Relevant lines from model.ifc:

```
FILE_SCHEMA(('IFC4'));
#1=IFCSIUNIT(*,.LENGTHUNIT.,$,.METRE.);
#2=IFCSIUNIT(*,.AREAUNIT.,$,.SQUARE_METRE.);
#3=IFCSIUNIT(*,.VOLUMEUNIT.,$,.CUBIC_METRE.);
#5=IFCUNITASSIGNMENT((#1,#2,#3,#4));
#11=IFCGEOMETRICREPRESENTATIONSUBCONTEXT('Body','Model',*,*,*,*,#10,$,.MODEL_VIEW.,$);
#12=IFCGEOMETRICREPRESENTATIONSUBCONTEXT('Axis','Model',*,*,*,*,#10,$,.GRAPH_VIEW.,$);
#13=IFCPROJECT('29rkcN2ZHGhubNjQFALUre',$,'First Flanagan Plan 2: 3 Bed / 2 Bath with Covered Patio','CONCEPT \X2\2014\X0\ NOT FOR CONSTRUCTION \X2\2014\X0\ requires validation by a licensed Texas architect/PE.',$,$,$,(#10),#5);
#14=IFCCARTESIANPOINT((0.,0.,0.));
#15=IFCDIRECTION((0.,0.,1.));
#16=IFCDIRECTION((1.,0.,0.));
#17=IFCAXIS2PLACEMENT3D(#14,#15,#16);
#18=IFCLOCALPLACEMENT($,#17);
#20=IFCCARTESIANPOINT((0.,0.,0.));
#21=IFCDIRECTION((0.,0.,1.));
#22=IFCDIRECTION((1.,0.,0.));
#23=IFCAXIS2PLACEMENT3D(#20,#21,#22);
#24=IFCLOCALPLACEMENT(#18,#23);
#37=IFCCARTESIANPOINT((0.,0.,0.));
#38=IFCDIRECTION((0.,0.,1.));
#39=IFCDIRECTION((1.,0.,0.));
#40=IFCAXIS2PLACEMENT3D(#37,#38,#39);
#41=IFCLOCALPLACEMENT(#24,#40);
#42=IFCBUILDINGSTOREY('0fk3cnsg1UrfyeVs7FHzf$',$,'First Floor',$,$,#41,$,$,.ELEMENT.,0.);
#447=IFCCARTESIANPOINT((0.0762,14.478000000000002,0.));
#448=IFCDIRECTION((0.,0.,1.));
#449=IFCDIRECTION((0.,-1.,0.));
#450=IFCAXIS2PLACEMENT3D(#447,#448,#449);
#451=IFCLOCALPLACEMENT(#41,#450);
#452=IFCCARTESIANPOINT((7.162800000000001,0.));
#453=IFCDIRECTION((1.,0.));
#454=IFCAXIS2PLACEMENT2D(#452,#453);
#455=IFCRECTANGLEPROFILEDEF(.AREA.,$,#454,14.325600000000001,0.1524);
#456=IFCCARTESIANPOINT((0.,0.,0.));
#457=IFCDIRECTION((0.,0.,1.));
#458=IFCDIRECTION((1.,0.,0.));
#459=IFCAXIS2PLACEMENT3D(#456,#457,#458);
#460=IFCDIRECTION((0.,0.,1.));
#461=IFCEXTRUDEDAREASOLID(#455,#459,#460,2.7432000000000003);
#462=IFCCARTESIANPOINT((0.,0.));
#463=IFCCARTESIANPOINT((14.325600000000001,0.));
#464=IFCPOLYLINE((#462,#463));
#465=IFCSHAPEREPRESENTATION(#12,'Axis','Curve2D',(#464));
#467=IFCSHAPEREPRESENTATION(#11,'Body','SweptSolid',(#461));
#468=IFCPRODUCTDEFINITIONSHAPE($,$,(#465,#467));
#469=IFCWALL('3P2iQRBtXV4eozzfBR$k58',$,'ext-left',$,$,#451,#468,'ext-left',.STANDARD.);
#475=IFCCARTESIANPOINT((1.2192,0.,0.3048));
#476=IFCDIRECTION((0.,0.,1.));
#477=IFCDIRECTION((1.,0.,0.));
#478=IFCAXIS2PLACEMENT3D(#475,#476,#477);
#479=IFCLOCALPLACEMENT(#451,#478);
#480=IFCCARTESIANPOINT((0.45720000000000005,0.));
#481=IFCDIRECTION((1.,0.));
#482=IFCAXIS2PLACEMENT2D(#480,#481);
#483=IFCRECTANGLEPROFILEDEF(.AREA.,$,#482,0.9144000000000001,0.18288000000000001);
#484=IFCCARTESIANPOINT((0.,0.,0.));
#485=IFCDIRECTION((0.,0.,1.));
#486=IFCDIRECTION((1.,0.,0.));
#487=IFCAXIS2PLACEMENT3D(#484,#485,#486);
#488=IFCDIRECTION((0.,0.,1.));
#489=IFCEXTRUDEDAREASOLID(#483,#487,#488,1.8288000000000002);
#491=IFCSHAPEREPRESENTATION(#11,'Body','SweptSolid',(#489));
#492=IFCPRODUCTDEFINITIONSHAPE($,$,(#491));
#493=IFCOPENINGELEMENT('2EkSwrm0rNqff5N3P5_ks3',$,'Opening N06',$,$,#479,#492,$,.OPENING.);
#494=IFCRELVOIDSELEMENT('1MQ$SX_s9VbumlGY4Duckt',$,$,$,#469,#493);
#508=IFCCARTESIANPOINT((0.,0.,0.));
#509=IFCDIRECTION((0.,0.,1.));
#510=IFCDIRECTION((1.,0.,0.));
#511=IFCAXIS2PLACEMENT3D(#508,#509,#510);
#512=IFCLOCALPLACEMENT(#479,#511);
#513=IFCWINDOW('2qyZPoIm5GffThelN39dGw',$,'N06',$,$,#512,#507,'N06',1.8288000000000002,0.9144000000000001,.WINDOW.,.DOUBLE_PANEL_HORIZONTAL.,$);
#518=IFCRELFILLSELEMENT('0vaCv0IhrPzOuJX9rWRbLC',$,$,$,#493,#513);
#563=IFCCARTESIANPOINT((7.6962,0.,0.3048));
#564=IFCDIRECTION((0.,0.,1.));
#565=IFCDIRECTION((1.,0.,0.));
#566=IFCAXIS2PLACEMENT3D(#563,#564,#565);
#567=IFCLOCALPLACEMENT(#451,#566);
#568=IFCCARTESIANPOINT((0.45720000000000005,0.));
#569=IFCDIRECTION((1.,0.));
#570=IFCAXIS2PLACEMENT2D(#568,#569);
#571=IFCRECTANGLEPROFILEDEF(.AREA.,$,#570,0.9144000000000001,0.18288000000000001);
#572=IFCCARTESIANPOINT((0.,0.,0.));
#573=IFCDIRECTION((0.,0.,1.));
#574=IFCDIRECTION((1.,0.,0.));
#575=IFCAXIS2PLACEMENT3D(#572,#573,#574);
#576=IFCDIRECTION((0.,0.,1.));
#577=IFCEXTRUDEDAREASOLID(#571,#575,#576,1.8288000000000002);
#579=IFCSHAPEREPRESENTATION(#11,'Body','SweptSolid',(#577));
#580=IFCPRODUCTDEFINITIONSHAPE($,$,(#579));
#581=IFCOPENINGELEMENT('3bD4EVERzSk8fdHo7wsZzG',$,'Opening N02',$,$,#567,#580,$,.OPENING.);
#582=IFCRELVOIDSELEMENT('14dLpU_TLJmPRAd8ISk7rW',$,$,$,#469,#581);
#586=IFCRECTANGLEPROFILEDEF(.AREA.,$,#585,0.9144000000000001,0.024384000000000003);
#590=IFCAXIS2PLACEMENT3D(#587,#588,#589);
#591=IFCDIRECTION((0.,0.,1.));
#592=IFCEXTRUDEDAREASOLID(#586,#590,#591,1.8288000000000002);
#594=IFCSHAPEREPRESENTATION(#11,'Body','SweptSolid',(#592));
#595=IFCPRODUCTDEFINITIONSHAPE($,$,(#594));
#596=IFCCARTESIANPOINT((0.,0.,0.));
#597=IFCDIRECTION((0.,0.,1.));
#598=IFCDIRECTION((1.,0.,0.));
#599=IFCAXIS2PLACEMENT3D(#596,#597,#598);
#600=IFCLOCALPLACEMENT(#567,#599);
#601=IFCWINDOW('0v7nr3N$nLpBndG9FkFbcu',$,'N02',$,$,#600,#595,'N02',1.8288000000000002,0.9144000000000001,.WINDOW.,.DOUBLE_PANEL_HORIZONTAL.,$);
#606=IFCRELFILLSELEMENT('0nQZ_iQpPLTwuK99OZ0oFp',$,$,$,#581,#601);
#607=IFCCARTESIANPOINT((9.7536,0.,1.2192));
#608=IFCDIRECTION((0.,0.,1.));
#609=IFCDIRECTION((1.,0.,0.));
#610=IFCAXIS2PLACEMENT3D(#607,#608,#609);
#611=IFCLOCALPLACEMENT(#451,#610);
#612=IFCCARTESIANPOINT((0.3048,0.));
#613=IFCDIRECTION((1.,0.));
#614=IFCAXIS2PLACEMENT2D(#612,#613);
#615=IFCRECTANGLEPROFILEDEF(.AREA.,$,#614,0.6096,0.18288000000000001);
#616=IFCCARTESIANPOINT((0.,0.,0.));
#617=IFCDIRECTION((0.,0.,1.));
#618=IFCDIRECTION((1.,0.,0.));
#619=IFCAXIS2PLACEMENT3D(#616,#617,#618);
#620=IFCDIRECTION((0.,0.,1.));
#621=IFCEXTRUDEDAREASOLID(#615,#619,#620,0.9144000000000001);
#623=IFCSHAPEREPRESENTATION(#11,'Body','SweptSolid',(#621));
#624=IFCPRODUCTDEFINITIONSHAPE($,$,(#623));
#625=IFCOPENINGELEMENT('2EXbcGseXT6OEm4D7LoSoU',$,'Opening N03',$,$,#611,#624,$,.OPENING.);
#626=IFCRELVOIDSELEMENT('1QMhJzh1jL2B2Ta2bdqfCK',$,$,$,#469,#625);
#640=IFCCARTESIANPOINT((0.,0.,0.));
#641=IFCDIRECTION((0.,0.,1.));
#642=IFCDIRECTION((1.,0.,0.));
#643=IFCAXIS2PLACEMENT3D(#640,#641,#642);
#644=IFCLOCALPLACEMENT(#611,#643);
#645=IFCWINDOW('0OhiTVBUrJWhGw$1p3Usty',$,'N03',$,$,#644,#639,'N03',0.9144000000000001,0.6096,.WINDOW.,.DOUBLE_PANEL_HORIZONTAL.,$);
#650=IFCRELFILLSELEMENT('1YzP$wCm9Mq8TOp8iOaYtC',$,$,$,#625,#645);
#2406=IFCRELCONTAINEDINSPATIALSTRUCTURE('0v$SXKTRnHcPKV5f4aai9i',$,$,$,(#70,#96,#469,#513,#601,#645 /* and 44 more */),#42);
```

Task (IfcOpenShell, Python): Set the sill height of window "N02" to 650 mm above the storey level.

```python
import numpy as np
import ifcopenshell
import ifcopenshell.api.geometry
import ifcopenshell.geom
import ifcopenshell.util.element
import ifcopenshell.util.placement
import ifcopenshell.util.shape
import ifcopenshell.util.unit

model = ifcopenshell.open("model.ifc")
unit_scale = ifcopenshell.util.unit.calculate_unit_scale(model)

window = model.by_id(601)
opening = window.FillsVoids[0].RelatingOpeningElement
storey = ifcopenshell.util.element.get_container(window, ifc_class="IfcBuildingStorey")
level = ifcopenshell.util.placement.get_local_placement(storey.ObjectPlacement)[2, 3]

# The opening's origin need not be at the sill, so measure its lowest point.
shape = ifcopenshell.geom.create_shape(ifcopenshell.geom.settings(), opening)
bottom = ifcopenshell.util.shape.get_shape_bottom_elevation(shape, shape.geometry) / unit_scale
dz = level + 0.65 / unit_scale - bottom

shift = np.array([0.0, 0.0, dz])
# The window is placed relative to its opening, so it follows when the opening moves.
matrix = ifcopenshell.util.placement.get_local_placement(opening.ObjectPlacement)
matrix[:3, 3] += shift
ifcopenshell.api.geometry.edit_object_placement(
    model, product=opening, matrix=matrix, is_si=False, should_transform_children=True
)

print(f"moved by {dz * unit_scale:+.3f} m")

model.write("model_updated.ifc")
```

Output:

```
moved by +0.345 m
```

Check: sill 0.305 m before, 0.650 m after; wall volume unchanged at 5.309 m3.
